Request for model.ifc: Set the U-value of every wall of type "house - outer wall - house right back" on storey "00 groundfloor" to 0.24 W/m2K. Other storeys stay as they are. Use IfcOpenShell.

First a look at what the model holds.

```python
import ifcopenshell
import ifcopenshell.util.element

model = ifcopenshell.open("model.ifc")
print(model.schema)
storey = next(s for s in model.by_type("IfcBuildingStorey") if s.Name == "00 groundfloor")
walls = [e for e in ifcopenshell.util.element.get_decomposition(storey) if e.is_a("IfcWall")]
seen = {}
for e in walls:
    element_type = ifcopenshell.util.element.get_type(e)
    key = (element_type.Name if element_type != e and element_type else None, ifcopenshell.util.element.get_pset(e, "Pset_WallCommon", "ThermalTransmittance"))
    seen[key] = seen.get(key, 0) + 1
for (name, value), count in sorted(seen.items(), key=str):
    print(count, "x", name, "|", value)
```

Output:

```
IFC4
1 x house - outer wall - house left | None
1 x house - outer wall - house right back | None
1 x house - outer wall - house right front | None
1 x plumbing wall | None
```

```python
import ifcopenshell
import ifcopenshell.api.pset
import ifcopenshell.util.element

model = ifcopenshell.open("model.ifc")

storey = next(s for s in model.by_type("IfcBuildingStorey") if s.Name == "00 groundfloor")
walls = [e for e in ifcopenshell.util.element.get_decomposition(storey) if e.is_a("IfcWall")]

count = 0
for e in walls:
    element_type = ifcopenshell.util.element.get_type(e)
    if element_type in (None, e) or element_type.Name != "house - outer wall - house right back":
        continue
    # add_pset returns the element's existing set when there is one.
    pset = ifcopenshell.api.pset.add_pset(model, product=e, name="Pset_WallCommon")
    ifcopenshell.api.pset.edit_pset(model, pset=pset, properties={"ThermalTransmittance": 0.24})
    count += 1

print(count, "walls updated")

model.write("model_edited.ifc")
```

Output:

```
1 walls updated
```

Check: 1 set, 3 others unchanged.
